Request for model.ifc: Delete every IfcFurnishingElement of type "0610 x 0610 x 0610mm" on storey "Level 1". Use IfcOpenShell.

First a look at what the model holds.

```python
import ifcopenshell
import ifcopenshell.util.element

model = ifcopenshell.open("model.ifc")
print(model.schema)
storey = next(s for s in model.by_type("IfcBuildingStorey") if s.Name == "Level 1")
furniture = [e for e in ifcopenshell.util.element.get_decomposition(storey) if e.is_a("IfcFurnishingElement")]
seen = {}
for e in furniture:
    element_type = ifcopenshell.util.element.get_type(e)
    name = element_type.Name if element_type not in (None, e) else None
    seen[name] = seen.get(name, 0) + 1
for name, count in sorted(seen.items(), key=str):
    print(count, "x", name)
```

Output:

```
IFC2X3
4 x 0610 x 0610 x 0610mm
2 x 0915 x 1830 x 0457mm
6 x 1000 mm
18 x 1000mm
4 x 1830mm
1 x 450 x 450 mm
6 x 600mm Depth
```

```python
import ifcopenshell
import ifcopenshell.api.root
import ifcopenshell.util.element

model = ifcopenshell.open("model.ifc")

storey = next(s for s in model.by_type("IfcBuildingStorey") if s.Name == "Level 1")
furniture = [e for e in ifcopenshell.util.element.get_decomposition(storey) if e.is_a("IfcFurnishingElement")]
targets = [e for e in furniture if (t := ifcopenshell.util.element.get_type(e)) not in (None, e) and t.Name == "0610 x 0610 x 0610mm"]

for e in targets:
    ifcopenshell.api.root.remove_product(model, product=e)
print(len(targets), "removed")

model.write("model_v2.ifc")
```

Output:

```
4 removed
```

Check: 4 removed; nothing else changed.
